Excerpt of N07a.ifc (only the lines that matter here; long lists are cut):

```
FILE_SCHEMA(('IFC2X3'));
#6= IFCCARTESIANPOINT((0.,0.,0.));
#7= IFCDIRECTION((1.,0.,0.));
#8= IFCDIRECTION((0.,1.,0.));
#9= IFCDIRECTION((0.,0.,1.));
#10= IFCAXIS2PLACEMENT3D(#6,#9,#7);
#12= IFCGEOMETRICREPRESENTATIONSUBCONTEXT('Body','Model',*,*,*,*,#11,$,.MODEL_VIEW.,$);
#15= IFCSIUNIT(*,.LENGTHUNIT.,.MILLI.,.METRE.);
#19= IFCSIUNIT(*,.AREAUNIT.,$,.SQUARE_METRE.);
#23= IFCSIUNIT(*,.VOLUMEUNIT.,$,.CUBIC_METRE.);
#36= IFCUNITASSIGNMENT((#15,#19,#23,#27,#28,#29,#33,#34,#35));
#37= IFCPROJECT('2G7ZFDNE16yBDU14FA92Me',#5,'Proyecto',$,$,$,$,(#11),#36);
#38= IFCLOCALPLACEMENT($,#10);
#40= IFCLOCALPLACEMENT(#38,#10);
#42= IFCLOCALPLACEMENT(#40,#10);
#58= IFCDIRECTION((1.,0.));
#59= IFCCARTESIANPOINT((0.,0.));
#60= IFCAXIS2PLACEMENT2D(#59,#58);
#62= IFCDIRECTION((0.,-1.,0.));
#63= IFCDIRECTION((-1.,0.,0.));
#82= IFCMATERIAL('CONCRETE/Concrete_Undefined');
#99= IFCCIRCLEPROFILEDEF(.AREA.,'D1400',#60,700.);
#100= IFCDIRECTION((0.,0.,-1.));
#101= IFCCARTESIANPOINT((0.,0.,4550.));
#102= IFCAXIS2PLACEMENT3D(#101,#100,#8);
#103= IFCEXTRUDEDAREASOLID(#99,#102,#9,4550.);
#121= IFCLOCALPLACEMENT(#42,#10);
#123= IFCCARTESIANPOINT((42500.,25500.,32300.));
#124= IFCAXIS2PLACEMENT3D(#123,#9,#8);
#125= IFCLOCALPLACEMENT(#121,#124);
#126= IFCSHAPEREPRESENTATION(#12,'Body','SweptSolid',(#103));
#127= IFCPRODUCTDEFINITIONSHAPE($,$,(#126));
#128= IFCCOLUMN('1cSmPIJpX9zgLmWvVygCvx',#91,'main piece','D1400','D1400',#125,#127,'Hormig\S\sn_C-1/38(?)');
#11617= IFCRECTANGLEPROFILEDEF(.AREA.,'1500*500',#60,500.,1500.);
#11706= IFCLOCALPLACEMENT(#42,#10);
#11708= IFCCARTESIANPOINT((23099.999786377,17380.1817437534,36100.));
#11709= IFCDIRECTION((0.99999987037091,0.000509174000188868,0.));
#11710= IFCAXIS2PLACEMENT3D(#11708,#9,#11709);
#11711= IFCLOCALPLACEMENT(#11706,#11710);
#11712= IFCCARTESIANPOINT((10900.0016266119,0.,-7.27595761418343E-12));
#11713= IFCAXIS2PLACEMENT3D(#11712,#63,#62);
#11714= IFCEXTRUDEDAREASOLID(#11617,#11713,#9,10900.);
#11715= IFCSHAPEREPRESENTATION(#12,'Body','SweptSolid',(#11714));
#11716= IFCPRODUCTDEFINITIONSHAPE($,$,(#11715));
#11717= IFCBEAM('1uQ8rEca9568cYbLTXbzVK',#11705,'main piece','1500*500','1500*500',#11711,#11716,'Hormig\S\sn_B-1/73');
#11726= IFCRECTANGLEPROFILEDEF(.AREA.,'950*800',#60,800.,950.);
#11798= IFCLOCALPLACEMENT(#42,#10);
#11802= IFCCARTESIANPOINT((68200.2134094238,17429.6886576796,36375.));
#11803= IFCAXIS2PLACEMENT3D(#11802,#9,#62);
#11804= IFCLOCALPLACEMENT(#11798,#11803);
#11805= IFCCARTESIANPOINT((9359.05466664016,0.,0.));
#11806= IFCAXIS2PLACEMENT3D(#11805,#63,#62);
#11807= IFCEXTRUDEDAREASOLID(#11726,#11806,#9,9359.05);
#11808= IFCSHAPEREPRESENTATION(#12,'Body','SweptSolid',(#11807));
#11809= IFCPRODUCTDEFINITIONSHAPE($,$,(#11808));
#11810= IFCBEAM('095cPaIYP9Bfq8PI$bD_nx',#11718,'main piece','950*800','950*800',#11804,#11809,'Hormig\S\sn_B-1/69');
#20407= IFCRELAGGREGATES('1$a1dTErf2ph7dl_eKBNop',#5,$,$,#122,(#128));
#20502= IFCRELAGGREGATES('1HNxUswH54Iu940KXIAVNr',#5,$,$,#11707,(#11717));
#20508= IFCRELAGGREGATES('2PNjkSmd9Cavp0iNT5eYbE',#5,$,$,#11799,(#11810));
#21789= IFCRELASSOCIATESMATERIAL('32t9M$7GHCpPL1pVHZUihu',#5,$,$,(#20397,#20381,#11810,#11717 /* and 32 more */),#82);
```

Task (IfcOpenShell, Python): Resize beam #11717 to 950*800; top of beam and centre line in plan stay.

```python
import ifcopenshell
import ifcopenshell.util.element
import ifcopenshell.util.representation

model = ifcopenshell.open("N07a.ifc")

member = model.by_id(11717)
source = next(p for p in model.by_type("IfcRectangleProfileDef") if p.ProfileName == "950*800")

body = ifcopenshell.util.representation.get_representation(member, "Model", "Body")
solid = body.Items[0]
old_profile = solid.SweptArea

# Copy the section's sizes but keep this member's own profile position.
profile = ifcopenshell.util.element.copy(model, source)
# Profiles are centred, so shift by half the change in depth to hold the top.
shift = (old_profile.YDim - profile.YDim) / 2
x, y = old_profile.Position.Location.Coordinates
up = (0.0, 1.0)  # upwards, in the solid's own plane
location = model.createIfcCartesianPoint((x + up[0] * shift, y + up[1] * shift))
profile.Position = model.createIfcAxis2Placement2D(location, old_profile.Position.RefDirection)
solid.SweptArea = profile
if not model.get_total_inverses(old_profile):
    ifcopenshell.util.element.remove_deep2(model, old_profile)
member.Description = member.Description.replace("1500*500", "950*800")
member.ObjectType = member.ObjectType.replace("1500*500", "950*800")

print(solid.SweptArea)

model.write("N07a_v2.ifc")
```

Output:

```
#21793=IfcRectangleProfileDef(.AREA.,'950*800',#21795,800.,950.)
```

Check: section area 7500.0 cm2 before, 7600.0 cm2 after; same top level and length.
